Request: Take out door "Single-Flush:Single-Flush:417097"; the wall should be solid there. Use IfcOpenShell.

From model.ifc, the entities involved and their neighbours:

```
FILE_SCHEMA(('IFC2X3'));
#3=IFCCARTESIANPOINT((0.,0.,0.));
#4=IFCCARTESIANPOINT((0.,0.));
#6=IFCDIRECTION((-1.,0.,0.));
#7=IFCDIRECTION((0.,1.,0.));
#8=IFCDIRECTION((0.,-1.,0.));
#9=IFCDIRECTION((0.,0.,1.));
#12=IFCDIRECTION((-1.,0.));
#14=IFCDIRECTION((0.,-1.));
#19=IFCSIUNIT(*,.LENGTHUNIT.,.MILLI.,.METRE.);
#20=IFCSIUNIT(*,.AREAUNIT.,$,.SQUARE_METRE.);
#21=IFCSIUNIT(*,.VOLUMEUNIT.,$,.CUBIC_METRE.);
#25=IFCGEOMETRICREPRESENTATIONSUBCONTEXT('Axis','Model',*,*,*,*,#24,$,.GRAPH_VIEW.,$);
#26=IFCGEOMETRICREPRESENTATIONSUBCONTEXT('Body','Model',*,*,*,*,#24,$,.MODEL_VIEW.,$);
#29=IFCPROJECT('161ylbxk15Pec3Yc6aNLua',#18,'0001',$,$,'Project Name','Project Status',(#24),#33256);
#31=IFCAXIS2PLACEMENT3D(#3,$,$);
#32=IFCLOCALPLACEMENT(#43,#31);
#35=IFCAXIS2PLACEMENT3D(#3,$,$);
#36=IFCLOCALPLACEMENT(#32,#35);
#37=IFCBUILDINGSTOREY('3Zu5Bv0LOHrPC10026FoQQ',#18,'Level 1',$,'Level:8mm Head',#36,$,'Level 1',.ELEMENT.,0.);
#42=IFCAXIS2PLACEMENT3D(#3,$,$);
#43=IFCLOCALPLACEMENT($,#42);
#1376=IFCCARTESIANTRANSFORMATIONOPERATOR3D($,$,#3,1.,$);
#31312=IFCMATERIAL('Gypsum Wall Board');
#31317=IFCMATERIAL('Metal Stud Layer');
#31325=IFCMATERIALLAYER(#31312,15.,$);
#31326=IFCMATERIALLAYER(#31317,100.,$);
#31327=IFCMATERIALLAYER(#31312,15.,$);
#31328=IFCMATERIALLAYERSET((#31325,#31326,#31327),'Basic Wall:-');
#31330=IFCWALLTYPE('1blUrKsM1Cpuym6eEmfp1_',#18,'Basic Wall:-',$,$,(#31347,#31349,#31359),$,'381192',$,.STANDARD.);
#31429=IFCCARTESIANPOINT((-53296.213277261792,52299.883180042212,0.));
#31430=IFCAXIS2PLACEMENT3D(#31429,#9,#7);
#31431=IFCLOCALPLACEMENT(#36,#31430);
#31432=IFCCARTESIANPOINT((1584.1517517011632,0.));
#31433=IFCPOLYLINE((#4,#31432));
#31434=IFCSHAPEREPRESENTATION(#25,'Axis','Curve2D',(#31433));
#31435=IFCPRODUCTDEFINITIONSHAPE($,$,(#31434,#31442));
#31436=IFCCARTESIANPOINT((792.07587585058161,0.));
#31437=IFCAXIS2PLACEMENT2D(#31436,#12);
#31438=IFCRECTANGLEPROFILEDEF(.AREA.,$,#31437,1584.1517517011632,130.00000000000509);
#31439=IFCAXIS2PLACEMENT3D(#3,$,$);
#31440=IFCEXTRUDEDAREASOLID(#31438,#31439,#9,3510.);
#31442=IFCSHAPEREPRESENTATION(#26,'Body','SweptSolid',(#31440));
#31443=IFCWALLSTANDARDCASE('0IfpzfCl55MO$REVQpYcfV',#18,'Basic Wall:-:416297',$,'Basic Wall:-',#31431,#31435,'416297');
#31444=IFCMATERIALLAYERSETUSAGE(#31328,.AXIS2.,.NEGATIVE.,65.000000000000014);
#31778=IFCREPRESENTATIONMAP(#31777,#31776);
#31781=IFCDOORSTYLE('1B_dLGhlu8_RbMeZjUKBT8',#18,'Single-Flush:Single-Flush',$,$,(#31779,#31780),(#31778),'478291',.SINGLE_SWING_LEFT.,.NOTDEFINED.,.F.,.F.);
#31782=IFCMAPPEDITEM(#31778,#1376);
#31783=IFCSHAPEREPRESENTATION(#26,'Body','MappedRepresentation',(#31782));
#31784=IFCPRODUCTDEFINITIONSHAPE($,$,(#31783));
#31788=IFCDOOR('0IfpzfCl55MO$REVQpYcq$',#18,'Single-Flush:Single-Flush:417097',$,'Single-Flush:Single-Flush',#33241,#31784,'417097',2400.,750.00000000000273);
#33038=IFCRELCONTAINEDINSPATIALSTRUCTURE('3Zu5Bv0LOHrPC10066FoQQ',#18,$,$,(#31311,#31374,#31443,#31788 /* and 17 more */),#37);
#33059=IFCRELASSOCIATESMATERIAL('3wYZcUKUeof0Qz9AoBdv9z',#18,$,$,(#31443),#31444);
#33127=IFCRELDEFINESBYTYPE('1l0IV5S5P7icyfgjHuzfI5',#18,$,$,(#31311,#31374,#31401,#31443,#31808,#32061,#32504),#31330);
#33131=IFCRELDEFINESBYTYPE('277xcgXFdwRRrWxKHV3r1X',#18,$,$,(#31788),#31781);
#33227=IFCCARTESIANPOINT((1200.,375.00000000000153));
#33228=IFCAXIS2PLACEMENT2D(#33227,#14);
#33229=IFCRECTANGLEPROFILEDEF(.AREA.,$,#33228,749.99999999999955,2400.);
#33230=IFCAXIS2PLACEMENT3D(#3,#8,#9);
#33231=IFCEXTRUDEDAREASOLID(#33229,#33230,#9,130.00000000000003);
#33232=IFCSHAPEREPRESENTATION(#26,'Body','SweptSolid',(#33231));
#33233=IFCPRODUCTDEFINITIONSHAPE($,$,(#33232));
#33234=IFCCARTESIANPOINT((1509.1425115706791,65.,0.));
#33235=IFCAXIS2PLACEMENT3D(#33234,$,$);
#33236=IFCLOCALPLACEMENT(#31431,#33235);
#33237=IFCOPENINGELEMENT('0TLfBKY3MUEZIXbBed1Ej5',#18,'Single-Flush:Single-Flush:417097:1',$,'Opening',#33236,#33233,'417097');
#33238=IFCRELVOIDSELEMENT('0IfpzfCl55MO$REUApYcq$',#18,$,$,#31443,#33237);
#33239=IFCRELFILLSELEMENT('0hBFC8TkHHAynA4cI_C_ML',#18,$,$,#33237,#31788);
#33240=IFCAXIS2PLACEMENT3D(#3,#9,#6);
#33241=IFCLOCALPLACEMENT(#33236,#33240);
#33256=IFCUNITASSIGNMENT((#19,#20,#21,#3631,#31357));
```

```python
import ifcopenshell
import ifcopenshell.api.feature
import ifcopenshell.api.root
import ifcopenshell.geom
import ifcopenshell.util.shape

model = ifcopenshell.open("model.ifc")
settings = ifcopenshell.geom.settings()


def volume(element):
    """Net volume in cubic metres, openings subtracted."""
    shape = ifcopenshell.geom.create_shape(settings, element)
    return ifcopenshell.util.shape.get_volume(shape.geometry)


door = model.by_guid("0IfpzfCl55MO$REVQpYcq$")
opening = door.FillsVoids[0].RelatingOpeningElement
wall = opening.VoidsElements[0].RelatingBuildingElement
before = volume(wall)

ifcopenshell.api.root.remove_product(model, product=door)
ifcopenshell.api.feature.remove_feature(model, feature=opening)

after = volume(wall)

print(f"wall volume {before:.3f} -> {after:.3f} m3")

model.write("model_updated.ifc")
```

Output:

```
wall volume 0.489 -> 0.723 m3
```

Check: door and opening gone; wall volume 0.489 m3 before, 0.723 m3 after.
